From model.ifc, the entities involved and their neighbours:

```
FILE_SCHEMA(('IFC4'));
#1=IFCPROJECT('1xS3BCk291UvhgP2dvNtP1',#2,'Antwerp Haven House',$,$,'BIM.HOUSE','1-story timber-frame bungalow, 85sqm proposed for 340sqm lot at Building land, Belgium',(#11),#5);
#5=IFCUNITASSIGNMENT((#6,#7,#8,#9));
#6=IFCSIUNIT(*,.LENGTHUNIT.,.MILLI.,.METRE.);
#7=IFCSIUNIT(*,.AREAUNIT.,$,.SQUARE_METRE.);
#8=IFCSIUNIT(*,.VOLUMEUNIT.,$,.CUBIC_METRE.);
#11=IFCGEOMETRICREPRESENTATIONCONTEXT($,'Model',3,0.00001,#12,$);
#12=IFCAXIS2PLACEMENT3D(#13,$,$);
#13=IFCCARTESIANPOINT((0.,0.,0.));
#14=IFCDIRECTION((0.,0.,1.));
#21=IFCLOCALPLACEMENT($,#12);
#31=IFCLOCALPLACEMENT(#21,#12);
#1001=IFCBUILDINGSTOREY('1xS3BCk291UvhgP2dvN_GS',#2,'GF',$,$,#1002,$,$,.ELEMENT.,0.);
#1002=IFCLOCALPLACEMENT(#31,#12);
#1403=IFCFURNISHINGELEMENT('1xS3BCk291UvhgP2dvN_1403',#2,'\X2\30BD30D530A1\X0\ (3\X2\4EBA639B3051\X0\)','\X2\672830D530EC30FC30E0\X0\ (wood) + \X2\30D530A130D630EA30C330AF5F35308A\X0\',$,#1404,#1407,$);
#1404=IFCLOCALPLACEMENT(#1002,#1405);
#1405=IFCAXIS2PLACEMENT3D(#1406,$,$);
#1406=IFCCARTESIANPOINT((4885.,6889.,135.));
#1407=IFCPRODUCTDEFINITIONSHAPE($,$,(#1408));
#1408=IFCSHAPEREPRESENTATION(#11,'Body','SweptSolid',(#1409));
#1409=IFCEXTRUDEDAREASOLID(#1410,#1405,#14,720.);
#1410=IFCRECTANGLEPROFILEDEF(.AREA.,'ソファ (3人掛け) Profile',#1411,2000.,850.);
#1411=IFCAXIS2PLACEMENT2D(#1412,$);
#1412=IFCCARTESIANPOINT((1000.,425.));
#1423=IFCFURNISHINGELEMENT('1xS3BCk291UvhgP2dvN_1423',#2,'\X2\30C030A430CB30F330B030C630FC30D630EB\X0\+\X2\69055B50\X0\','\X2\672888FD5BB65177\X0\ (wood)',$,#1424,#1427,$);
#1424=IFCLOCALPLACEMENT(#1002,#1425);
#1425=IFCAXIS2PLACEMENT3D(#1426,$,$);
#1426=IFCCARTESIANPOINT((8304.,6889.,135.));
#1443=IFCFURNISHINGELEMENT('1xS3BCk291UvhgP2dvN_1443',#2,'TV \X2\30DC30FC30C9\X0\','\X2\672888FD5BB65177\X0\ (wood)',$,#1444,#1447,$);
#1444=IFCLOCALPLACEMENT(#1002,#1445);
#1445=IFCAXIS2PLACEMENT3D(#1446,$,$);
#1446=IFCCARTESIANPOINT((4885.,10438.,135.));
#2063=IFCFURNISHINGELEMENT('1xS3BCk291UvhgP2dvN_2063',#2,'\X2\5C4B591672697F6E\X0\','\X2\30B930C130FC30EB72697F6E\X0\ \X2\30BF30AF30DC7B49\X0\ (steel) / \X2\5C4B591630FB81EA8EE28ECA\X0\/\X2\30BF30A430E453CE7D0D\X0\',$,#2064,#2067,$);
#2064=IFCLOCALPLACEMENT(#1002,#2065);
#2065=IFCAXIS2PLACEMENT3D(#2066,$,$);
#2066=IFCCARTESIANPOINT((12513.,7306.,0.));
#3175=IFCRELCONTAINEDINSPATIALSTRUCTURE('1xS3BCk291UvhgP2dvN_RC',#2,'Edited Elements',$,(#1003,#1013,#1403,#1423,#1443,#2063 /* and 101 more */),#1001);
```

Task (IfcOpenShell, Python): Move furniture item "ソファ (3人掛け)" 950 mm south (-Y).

```python
import ifcopenshell
import ifcopenshell.api.geometry
import ifcopenshell.util.placement
import ifcopenshell.util.unit

model = ifcopenshell.open("model.ifc")
unit_scale = ifcopenshell.util.unit.calculate_unit_scale(model)

item = model.by_guid("1xS3BCk291UvhgP2dvN_1403")
matrix = ifcopenshell.util.placement.get_local_placement(item.ObjectPlacement)
matrix[1, 3] -= 0.95 / unit_scale
ifcopenshell.api.geometry.edit_object_placement(model, product=item, matrix=matrix, is_si=False)

print(ifcopenshell.util.placement.get_local_placement(item.ObjectPlacement).round(3) + 0.0)

model.write("model_v2.ifc")
```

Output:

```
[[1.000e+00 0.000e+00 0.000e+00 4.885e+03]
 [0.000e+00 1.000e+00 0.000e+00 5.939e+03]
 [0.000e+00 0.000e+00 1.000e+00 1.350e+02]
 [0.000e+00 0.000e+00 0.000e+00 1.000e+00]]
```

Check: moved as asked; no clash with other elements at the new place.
